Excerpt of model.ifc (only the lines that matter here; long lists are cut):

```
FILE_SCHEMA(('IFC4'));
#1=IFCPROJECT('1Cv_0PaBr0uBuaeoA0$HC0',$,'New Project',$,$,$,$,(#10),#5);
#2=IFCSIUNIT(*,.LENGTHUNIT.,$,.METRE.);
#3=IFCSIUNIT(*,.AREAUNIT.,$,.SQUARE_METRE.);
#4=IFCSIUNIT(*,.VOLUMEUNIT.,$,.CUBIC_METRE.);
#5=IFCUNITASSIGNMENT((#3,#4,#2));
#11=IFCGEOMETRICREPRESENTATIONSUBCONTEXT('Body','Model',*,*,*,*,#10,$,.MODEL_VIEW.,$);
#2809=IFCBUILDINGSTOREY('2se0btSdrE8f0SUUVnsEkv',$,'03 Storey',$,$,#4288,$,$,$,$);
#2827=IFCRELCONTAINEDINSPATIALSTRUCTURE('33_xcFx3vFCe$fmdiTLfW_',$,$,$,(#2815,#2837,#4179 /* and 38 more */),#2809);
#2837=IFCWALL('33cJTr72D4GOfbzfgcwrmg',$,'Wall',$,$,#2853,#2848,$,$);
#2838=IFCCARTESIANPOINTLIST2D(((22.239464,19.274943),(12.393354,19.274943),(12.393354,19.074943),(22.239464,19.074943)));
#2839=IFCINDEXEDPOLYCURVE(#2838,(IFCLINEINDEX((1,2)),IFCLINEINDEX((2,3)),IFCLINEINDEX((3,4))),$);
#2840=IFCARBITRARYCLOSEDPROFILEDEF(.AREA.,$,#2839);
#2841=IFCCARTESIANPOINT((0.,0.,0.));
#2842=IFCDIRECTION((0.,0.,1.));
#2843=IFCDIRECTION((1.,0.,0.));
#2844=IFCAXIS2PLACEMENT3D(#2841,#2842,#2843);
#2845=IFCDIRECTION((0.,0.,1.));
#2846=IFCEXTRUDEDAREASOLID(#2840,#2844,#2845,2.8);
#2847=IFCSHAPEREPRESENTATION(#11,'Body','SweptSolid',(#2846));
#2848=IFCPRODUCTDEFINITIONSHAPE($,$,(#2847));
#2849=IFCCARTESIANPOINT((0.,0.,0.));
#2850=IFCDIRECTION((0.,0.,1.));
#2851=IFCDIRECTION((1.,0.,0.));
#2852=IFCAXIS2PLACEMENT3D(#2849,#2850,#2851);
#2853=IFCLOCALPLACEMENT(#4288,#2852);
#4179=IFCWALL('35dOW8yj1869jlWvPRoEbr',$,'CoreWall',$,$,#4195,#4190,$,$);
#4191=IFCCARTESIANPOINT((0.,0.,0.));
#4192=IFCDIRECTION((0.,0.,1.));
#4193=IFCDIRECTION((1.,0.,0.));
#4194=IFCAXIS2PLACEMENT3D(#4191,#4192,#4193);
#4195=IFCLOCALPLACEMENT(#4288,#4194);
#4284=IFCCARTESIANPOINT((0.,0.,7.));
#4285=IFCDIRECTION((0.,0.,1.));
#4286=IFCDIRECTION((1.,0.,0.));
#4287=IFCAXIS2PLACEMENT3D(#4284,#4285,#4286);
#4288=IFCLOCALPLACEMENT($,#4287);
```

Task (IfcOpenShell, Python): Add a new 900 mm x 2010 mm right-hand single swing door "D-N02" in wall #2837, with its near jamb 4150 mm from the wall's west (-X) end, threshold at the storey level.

```python
import numpy as np
import ifcopenshell
import ifcopenshell.api.feature
import ifcopenshell.api.geometry
import ifcopenshell.api.root
import ifcopenshell.api.spatial
import ifcopenshell.geom
import ifcopenshell.util.element
import ifcopenshell.util.placement
import ifcopenshell.util.representation
import ifcopenshell.util.shape
import ifcopenshell.util.unit

model = ifcopenshell.open("model.ifc")
unit_scale = ifcopenshell.util.unit.calculate_unit_scale(model)
settings = ifcopenshell.geom.settings()


def volume(element):
    """Net volume in cubic metres, openings subtracted."""
    shape = ifcopenshell.geom.create_shape(settings, element)
    return ifcopenshell.util.shape.get_volume(shape.geometry)


wall = model.by_id(2837)
storey = ifcopenshell.util.element.get_container(wall, ifc_class="IfcBuildingStorey")
context = ifcopenshell.util.representation.get_context(model, "Model", "Body", "MODEL_VIEW")
before = volume(wall)

width, height, from_end, sill = 0.9, 2.01, 4.15, 0.0  # metres

# The wall runs along its own X axis, and the end named is its -X end.
wall_shape = ifcopenshell.geom.create_shape(settings, wall)
x, y, z = ifcopenshell.util.shape.get_vertices(wall_shape.geometry).T
start = x.min() + from_end
face, thickness = float(y.min()), float(y.max() - y.min())
wall_matrix = ifcopenshell.util.placement.get_local_placement(wall.ObjectPlacement)
level = ifcopenshell.util.placement.get_local_placement(storey.ObjectPlacement)[2, 3]


def in_wall(x, y):
    """Placement at x, y metres in the wall's axes, at sill height."""
    matrix = wall_matrix.copy()
    matrix[:, 3] = wall_matrix @ np.array([x / unit_scale, y / unit_scale, 0.0, 1.0])
    matrix[2, 3] = level + sill / unit_scale
    return matrix


# Opening: a box that overshoots both wall faces by 50 mm.
opening = ifcopenshell.api.root.create_entity(model, ifc_class="IfcOpeningElement", predefined_type="OPENING")
box = ifcopenshell.api.geometry.add_wall_representation(
    model, context=context, length=width, height=height, thickness=thickness + 0.1
)
ifcopenshell.api.geometry.assign_representation(model, product=opening, representation=box)
ifcopenshell.api.geometry.edit_object_placement(model, product=opening, matrix=in_wall(start, face - 0.05), is_si=False)
ifcopenshell.api.feature.add_feature(model, feature=opening, element=wall)

door = ifcopenshell.api.root.create_entity(model, ifc_class="IfcDoor", name="D-N02", predefined_type="DOOR")
door.OverallWidth, door.OverallHeight = width / unit_scale, height / unit_scale
door.OperationType = "SINGLE_SWING_RIGHT"
body = ifcopenshell.api.geometry.add_door_representation(
    model,
    context=context,
    overall_width=door.OverallWidth,
    overall_height=door.OverallHeight,
    operation_type="SINGLE_SWING_RIGHT",
    lining_properties={"LiningDepth": thickness / unit_scale, "ThresholdDepth": thickness / unit_scale},
)
ifcopenshell.api.geometry.assign_representation(model, product=door, representation=body)
ifcopenshell.api.spatial.assign_container(model, products=[door], relating_structure=storey)
ifcopenshell.api.feature.add_filling(model, opening=opening, element=door)

# The lining spans the wall, so the door starts at the wall face.
ifcopenshell.api.geometry.edit_object_placement(model, product=door, matrix=in_wall(start, face), is_si=False)

after = volume(wall)

print(f"wall volume {before:.3f} -> {after:.3f} m3")

model.write("model-out.ifc")
```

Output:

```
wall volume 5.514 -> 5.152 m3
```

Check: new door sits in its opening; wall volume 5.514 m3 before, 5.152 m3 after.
